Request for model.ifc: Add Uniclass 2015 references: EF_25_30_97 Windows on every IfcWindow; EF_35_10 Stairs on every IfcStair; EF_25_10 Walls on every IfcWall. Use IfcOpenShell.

First a look at what the model holds.

```python
import ifcopenshell

model = ifcopenshell.open("model.ifc")
print(model.schema)
print("classifications:", [c.Name for c in model.by_type("IfcClassification")])
for ifc_class in ("IfcDoor", "IfcRoof", "IfcStair", "IfcWall", "IfcWindow"):
    print(ifc_class, len(model.by_type(ifc_class)))
```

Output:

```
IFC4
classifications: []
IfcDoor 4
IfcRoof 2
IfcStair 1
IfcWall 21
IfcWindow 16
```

```python
import ifcopenshell
import ifcopenshell.api.classification

model = ifcopenshell.open("model.ifc")

system = ifcopenshell.api.classification.add_classification(model, classification="Uniclass 2015")

codes = {
    "IfcWindow": ("EF_25_30_97", "Windows"),
    "IfcStair": ("EF_35_10", "Stairs"),
    "IfcWall": ("EF_25_10", "Walls"),
}
for ifc_class, (code, name) in codes.items():
    products = model.by_type(ifc_class)
    ifcopenshell.api.classification.add_reference(
        model, products=products, classification=system, identification=code, name=name
    )
    print(code, len(products))

model.write("model_v2.ifc")
```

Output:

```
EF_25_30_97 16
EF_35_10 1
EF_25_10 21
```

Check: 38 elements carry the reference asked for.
